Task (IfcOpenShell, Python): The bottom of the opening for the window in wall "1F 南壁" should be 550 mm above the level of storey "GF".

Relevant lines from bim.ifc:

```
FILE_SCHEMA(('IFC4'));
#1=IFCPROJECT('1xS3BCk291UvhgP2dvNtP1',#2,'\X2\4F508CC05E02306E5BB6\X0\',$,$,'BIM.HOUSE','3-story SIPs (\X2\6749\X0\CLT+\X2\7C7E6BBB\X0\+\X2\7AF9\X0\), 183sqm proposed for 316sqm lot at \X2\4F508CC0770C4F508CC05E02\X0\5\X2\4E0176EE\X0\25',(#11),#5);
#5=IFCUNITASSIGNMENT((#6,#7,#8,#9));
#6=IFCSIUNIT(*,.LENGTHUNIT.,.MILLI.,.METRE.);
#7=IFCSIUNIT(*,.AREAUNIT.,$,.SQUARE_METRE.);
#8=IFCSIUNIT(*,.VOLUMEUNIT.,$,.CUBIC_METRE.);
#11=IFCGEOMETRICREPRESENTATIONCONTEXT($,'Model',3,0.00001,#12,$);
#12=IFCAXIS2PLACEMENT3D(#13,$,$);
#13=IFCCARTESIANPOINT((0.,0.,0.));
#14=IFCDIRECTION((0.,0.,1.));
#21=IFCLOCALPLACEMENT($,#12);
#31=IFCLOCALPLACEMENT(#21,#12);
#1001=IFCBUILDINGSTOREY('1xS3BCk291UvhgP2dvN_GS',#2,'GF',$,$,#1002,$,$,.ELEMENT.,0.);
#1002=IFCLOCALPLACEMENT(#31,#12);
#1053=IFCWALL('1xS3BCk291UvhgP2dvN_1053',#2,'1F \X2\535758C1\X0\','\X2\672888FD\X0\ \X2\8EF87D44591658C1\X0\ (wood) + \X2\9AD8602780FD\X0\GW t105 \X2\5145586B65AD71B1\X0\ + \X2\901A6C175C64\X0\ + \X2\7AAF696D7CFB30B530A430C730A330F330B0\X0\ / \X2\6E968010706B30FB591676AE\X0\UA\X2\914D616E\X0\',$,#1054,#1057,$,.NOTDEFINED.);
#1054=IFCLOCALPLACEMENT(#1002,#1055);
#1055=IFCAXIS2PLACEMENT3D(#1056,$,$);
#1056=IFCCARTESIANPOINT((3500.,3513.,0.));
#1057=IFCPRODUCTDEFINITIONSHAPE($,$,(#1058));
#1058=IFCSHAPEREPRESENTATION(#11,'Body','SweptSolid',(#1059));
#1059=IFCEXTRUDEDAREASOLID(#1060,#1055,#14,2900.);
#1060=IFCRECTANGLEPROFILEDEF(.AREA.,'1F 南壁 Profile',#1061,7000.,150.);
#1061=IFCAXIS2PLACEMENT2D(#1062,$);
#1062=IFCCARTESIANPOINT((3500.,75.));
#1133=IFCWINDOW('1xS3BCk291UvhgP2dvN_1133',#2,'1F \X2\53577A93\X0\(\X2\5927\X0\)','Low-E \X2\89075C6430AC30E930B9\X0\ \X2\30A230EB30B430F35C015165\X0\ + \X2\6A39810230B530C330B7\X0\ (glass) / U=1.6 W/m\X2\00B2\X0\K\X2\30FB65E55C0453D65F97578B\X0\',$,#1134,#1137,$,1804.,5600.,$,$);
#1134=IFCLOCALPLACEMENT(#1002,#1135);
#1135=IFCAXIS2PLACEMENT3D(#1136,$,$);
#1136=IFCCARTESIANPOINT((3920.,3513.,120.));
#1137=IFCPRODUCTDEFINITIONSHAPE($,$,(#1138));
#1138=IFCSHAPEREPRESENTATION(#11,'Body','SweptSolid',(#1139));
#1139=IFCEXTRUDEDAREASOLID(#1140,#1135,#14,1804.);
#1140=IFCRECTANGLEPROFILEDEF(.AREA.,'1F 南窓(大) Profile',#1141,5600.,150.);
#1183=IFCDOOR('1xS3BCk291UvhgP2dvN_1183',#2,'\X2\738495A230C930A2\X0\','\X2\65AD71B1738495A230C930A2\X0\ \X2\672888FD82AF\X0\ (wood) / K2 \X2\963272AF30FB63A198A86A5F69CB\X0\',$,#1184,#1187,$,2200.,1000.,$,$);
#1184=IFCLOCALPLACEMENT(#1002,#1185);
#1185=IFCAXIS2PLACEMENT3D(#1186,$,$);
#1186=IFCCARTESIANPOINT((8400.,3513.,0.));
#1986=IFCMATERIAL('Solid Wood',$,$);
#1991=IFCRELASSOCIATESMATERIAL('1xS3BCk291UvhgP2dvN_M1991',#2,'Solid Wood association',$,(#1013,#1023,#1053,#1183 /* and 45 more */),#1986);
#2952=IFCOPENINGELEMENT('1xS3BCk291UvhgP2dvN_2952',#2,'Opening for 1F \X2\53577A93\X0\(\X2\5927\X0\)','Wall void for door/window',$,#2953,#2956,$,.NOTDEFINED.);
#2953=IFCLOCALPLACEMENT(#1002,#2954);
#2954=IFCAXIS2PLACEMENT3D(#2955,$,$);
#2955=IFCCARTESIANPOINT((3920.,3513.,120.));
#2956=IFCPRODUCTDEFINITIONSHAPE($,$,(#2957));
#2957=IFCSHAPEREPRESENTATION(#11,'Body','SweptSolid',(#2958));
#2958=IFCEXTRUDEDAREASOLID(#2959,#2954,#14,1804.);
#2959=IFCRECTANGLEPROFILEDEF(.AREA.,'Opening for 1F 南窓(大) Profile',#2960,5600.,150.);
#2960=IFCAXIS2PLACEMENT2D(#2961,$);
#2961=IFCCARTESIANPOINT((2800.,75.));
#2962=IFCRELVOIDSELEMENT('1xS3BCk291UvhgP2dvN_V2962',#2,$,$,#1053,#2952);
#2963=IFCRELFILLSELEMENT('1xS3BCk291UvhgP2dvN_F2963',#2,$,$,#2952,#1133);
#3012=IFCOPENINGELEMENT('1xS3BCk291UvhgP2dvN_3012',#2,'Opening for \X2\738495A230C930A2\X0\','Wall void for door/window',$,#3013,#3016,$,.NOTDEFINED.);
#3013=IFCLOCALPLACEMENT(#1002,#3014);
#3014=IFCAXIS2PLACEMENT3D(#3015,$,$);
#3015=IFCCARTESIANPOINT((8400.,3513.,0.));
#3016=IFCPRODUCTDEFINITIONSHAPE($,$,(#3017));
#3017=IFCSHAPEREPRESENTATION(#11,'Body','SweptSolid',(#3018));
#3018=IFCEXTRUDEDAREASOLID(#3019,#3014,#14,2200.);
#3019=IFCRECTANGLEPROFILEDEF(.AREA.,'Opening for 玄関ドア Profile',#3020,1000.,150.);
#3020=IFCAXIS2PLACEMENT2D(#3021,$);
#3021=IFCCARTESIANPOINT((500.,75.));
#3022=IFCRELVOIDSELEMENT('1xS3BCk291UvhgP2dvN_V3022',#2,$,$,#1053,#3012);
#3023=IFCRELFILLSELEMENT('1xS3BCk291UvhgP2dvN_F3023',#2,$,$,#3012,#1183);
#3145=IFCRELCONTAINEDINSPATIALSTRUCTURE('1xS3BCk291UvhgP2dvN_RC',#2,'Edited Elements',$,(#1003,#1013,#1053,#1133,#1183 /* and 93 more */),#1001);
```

```python
import numpy as np
import ifcopenshell
import ifcopenshell.api.geometry
import ifcopenshell.geom
import ifcopenshell.util.element
import ifcopenshell.util.placement
import ifcopenshell.util.shape
import ifcopenshell.util.unit

model = ifcopenshell.open("bim.ifc")
unit_scale = ifcopenshell.util.unit.calculate_unit_scale(model)

window = model.by_guid("1xS3BCk291UvhgP2dvN_1133")
opening = window.FillsVoids[0].RelatingOpeningElement
storey = ifcopenshell.util.element.get_container(window, ifc_class="IfcBuildingStorey")
level = ifcopenshell.util.placement.get_local_placement(storey.ObjectPlacement)[2, 3]

# The opening's origin need not be at the sill, so measure its lowest point.
shape = ifcopenshell.geom.create_shape(ifcopenshell.geom.settings(), opening)
bottom = ifcopenshell.util.shape.get_shape_bottom_elevation(shape, shape.geometry) / unit_scale
dz = level + 0.55 / unit_scale - bottom

shift = np.array([0.0, 0.0, dz])
# The window is not placed relative to its opening, so move both.
for product in (opening, window):
    matrix = ifcopenshell.util.placement.get_local_placement(product.ObjectPlacement)
    matrix[:3, 3] += shift
    ifcopenshell.api.geometry.edit_object_placement(model, product=product, matrix=matrix, is_si=False)

print(f"moved by {dz * unit_scale:+.3f} m")

model.write("bim_updated.ifc")
```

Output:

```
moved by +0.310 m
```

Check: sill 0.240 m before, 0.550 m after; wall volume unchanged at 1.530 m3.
